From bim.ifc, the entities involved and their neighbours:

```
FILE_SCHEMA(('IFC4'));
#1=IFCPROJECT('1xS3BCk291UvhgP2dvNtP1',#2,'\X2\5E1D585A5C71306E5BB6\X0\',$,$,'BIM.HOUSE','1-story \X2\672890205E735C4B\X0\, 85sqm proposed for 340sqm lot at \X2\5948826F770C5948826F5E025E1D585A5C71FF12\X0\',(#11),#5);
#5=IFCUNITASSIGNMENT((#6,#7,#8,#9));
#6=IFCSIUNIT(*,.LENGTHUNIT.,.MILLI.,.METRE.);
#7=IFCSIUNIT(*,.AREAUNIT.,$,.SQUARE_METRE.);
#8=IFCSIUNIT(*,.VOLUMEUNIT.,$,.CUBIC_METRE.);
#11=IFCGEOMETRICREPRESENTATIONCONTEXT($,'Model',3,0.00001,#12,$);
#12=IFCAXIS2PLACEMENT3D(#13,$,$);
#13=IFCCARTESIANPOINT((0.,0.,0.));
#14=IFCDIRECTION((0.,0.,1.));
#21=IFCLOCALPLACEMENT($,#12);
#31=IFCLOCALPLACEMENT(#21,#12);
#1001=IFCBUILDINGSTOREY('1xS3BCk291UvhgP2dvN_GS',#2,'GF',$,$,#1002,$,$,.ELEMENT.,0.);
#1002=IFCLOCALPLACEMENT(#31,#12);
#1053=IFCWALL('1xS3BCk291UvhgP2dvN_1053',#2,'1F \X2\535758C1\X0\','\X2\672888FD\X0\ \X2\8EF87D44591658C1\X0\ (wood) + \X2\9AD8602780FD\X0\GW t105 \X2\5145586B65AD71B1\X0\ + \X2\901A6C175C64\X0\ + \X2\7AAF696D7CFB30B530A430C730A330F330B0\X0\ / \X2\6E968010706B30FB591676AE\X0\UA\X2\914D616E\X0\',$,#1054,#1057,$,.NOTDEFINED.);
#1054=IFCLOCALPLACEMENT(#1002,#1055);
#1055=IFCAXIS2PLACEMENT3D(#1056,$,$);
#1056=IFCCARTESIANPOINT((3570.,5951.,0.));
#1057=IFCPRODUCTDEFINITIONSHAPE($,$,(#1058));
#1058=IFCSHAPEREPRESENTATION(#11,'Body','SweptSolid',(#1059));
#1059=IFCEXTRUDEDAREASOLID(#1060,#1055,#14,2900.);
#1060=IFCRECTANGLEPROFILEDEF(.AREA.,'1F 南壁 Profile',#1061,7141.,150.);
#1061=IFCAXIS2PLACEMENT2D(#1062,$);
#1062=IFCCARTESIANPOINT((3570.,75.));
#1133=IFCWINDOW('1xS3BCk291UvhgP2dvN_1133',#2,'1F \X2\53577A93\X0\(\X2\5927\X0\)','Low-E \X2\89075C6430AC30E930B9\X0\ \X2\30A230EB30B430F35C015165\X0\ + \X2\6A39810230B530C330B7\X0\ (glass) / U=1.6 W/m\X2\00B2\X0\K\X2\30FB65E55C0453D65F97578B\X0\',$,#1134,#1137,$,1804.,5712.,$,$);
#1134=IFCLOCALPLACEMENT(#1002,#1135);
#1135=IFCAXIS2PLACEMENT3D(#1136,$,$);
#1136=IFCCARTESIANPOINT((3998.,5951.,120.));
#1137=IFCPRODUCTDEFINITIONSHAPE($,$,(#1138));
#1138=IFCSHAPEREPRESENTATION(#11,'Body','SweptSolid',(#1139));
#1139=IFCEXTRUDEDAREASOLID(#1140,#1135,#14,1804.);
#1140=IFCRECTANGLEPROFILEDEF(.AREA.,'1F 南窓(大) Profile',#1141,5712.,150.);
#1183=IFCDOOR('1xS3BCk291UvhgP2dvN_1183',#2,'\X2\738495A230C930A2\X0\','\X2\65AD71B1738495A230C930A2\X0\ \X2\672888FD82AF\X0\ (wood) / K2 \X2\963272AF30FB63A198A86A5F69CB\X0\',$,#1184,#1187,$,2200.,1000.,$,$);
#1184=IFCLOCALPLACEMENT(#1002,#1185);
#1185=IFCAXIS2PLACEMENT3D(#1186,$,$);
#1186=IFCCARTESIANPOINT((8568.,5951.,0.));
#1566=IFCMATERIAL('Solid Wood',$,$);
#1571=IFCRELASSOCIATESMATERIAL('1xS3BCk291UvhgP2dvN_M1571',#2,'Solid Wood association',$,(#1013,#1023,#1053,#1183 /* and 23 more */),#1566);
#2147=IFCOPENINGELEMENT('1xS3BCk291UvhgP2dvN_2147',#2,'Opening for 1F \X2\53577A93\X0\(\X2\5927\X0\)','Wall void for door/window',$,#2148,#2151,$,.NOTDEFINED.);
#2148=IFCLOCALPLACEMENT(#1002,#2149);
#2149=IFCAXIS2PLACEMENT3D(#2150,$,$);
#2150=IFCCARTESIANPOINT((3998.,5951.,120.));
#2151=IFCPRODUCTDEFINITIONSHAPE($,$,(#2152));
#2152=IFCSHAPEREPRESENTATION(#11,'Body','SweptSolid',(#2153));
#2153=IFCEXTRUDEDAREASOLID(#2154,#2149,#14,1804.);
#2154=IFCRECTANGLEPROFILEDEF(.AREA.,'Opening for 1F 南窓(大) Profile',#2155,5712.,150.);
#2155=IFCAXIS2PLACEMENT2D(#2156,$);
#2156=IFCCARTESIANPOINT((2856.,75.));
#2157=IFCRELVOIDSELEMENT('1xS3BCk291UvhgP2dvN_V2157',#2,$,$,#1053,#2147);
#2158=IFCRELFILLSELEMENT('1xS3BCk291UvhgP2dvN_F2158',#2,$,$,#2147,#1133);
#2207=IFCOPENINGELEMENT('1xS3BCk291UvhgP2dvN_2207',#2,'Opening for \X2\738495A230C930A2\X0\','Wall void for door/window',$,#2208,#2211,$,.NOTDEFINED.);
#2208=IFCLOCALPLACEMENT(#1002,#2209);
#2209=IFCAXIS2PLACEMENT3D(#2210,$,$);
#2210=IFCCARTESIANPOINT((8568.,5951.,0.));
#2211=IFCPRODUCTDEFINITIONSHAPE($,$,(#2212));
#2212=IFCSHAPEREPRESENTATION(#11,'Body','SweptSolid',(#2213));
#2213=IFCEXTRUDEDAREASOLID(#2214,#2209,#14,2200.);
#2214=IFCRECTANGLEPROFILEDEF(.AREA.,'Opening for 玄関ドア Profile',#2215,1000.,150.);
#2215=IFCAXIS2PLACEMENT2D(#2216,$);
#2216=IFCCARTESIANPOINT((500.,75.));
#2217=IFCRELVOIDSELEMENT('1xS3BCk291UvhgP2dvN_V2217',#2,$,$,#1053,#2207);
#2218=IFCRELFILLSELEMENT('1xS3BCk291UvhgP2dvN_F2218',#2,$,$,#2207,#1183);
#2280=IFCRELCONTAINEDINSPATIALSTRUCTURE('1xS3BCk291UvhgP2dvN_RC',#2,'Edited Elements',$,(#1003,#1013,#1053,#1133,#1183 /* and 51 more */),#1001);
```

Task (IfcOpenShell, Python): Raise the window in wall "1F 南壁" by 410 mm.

```python
import numpy as np
import ifcopenshell
import ifcopenshell.api.geometry
import ifcopenshell.util.placement
import ifcopenshell.util.unit

model = ifcopenshell.open("bim.ifc")
unit_scale = ifcopenshell.util.unit.calculate_unit_scale(model)

window = model.by_id(1133)
opening = window.FillsVoids[0].RelatingOpeningElement
dz = 0.41 / unit_scale

shift = np.array([0.0, 0.0, dz])
# The window is not placed relative to its opening, so move both.
for product in (opening, window):
    matrix = ifcopenshell.util.placement.get_local_placement(product.ObjectPlacement)
    matrix[:3, 3] += shift
    ifcopenshell.api.geometry.edit_object_placement(model, product=product, matrix=matrix, is_si=False)

print(f"moved by {dz * unit_scale:+.3f} m")

model.write("bim_edited.ifc")
```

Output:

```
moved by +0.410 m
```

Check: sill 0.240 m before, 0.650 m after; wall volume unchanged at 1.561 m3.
